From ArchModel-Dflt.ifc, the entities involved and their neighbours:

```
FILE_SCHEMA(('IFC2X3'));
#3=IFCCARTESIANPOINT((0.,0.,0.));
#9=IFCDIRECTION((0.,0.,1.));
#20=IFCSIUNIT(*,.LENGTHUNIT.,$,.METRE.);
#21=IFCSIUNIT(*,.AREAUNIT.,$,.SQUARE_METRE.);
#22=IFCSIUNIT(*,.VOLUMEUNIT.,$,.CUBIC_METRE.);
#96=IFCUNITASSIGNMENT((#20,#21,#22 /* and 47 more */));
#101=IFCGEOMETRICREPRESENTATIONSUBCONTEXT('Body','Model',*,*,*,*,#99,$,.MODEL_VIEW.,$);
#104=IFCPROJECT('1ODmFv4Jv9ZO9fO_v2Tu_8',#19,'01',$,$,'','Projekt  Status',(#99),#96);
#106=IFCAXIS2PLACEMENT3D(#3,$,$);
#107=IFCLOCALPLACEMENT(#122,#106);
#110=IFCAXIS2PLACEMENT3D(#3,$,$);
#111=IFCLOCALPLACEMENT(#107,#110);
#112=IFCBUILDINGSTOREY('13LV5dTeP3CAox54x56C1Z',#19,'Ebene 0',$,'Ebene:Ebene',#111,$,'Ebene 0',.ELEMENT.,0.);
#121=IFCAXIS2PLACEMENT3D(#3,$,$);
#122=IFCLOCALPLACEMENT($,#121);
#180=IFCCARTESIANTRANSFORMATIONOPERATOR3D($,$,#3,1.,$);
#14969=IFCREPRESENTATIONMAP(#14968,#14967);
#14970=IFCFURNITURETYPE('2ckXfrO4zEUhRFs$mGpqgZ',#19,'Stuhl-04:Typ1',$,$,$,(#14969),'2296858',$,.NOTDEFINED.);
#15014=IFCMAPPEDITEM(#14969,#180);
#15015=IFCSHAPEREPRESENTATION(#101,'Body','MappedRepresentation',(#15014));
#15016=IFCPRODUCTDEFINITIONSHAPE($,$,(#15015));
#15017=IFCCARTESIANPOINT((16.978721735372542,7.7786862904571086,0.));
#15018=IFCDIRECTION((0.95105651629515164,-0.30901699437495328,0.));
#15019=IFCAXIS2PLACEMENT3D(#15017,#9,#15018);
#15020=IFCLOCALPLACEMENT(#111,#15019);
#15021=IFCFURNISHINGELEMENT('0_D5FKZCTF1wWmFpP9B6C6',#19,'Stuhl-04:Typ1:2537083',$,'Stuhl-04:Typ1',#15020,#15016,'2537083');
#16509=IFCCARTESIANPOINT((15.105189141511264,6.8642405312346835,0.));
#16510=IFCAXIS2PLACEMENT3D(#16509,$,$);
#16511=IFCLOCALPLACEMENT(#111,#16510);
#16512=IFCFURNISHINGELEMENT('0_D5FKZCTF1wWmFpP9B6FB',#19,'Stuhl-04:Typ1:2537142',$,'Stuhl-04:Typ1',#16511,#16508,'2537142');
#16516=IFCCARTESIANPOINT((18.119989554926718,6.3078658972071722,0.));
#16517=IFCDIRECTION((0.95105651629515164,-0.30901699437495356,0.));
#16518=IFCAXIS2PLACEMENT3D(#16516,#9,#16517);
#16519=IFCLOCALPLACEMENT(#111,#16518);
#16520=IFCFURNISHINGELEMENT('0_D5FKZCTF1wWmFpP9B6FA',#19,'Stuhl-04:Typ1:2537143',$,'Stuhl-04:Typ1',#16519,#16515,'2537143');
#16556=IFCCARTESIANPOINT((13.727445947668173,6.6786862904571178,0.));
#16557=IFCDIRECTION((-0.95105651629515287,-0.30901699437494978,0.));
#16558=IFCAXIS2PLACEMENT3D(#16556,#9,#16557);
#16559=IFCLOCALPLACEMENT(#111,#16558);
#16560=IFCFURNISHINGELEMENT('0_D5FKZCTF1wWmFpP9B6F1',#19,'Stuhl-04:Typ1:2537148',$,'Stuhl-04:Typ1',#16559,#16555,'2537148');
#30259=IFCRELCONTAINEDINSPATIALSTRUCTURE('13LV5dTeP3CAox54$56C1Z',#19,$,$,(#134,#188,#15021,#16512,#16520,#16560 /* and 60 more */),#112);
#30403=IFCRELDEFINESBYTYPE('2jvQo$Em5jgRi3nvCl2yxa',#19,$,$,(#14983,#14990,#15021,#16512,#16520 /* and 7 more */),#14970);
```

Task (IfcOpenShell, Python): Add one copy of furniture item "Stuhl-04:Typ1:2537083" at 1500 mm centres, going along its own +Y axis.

```python
import ifcopenshell
import ifcopenshell.api.geometry
import ifcopenshell.api.root
import ifcopenshell.util.element
import ifcopenshell.util.placement
import ifcopenshell.util.unit

model = ifcopenshell.open("ArchModel-Dflt.ifc")
unit_scale = ifcopenshell.util.unit.calculate_unit_scale(model)

source = model.by_guid("0_D5FKZCTF1wWmFpP9B6C6")
base = ifcopenshell.util.placement.get_local_placement(source.ObjectPlacement)
step = base[:3, 1] * 1.5 / unit_scale

for i in range(1, 2):
    copy = ifcopenshell.api.root.copy_class(model, product=source)
    copy.Representation = ifcopenshell.util.element.copy_deep(
        model, source.Representation, exclude=["IfcGeometricRepresentationContext", "IfcRepresentationMap"]
    )
    copy.Name = "Stuhl-04:Typ1"
    copy.Tag = None
    matrix = base.copy()
    matrix[:3, 3] += i * step
    print("added at", matrix[:3, 3].round(3) + 0.0)
    ifcopenshell.api.geometry.edit_object_placement(model, product=copy, matrix=matrix, is_si=False)

model.write("ArchModel-Dflt_v2.ifc")
```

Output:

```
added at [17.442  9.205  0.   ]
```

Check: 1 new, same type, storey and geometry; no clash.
